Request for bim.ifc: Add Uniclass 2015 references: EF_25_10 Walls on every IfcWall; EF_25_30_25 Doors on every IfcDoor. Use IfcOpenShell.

First a look at what the model holds.

```python
import ifcopenshell

model = ifcopenshell.open("bim.ifc")
print(model.schema)
print("classifications:", [c.Name for c in model.by_type("IfcClassification")])
for ifc_class in ("IfcDoor", "IfcRoof", "IfcStair", "IfcWall", "IfcWindow"):
    print(ifc_class, len(model.by_type(ifc_class)))
```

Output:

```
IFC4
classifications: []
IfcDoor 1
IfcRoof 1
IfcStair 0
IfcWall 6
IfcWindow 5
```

```python
import ifcopenshell
import ifcopenshell.api.classification

model = ifcopenshell.open("bim.ifc")

system = ifcopenshell.api.classification.add_classification(model, classification="Uniclass 2015")

codes = {
    "IfcWall": ("EF_25_10", "Walls"),
    "IfcDoor": ("EF_25_30_25", "Doors"),
}
for ifc_class, (code, name) in codes.items():
    products = model.by_type(ifc_class)
    ifcopenshell.api.classification.add_reference(
        model, products=products, classification=system, identification=code, name=name
    )
    print(code, len(products))

model.write("bim_edited.ifc")
```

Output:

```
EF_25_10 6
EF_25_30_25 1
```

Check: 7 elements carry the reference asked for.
